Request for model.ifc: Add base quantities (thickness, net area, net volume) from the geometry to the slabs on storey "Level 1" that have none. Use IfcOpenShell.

First a look at what the model holds.

```python
import ifcopenshell
import ifcopenshell.util.element
import ifcopenshell.util.unit

model = ifcopenshell.open("model.ifc")
print(model.schema)
for unit_type in ("LENGTHUNIT", "AREAUNIT", "VOLUMEUNIT"):
    print(unit_type, ifcopenshell.util.unit.calculate_unit_scale(model, unit_type))
storey = next(s for s in model.by_type("IfcBuildingStorey") if s.Name == "Level 1")
slabs = [e for e in ifcopenshell.util.element.get_decomposition(storey) if e.is_a("IfcSlab")]
for e in sorted(slabs, key=lambda e: e.id()):
    print(e.id(), e.is_a(), e.Name, list(ifcopenshell.util.element.get_psets(e, qtos_only=True)), sep=" | ")
```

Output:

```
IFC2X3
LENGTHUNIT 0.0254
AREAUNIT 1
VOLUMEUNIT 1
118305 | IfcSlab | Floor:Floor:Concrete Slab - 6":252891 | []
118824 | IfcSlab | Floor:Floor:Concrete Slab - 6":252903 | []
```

```python
import ifcopenshell
import ifcopenshell.api.pset
import ifcopenshell.geom
import ifcopenshell.util.element
import ifcopenshell.util.shape
import ifcopenshell.util.unit

model = ifcopenshell.open("model.ifc")
unit_scale = ifcopenshell.util.unit.calculate_unit_scale(model)
area_scale = ifcopenshell.util.unit.calculate_unit_scale(model, "AREAUNIT")
volume_scale = ifcopenshell.util.unit.calculate_unit_scale(model, "VOLUMEUNIT")
settings = ifcopenshell.geom.settings()

storey = next(s for s in model.by_type("IfcBuildingStorey") if s.Name == "Level 1")
slabs = [e for e in ifcopenshell.util.element.get_decomposition(storey) if e.is_a("IfcSlab")]

for e in sorted(slabs, key=lambda e: e.id()):
    if ifcopenshell.util.element.get_psets(e, qtos_only=True, should_inherit=False):
        continue
    # Geometry comes back in metres, in the element's own axes.
    shape = ifcopenshell.geom.create_shape(settings, e)
    values = {
        "Width": ifcopenshell.util.shape.get_z(shape.geometry) / unit_scale,
        "NetArea": ifcopenshell.util.shape.get_footprint_area(shape.geometry) / area_scale,
        "NetVolume": ifcopenshell.util.shape.get_volume(shape.geometry) / volume_scale,
    }
    qto = ifcopenshell.api.pset.add_qto(model, product=e, name="BaseQuantities")
    ifcopenshell.api.pset.edit_qto(model, qto=qto, properties=values)
    print(e.id(), {k: round(v, 3) for k, v in values.items()})

model.write("model_rev.ifc")
```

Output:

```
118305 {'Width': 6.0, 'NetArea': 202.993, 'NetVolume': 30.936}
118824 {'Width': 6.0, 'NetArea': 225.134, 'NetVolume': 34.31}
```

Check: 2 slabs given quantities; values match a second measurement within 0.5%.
